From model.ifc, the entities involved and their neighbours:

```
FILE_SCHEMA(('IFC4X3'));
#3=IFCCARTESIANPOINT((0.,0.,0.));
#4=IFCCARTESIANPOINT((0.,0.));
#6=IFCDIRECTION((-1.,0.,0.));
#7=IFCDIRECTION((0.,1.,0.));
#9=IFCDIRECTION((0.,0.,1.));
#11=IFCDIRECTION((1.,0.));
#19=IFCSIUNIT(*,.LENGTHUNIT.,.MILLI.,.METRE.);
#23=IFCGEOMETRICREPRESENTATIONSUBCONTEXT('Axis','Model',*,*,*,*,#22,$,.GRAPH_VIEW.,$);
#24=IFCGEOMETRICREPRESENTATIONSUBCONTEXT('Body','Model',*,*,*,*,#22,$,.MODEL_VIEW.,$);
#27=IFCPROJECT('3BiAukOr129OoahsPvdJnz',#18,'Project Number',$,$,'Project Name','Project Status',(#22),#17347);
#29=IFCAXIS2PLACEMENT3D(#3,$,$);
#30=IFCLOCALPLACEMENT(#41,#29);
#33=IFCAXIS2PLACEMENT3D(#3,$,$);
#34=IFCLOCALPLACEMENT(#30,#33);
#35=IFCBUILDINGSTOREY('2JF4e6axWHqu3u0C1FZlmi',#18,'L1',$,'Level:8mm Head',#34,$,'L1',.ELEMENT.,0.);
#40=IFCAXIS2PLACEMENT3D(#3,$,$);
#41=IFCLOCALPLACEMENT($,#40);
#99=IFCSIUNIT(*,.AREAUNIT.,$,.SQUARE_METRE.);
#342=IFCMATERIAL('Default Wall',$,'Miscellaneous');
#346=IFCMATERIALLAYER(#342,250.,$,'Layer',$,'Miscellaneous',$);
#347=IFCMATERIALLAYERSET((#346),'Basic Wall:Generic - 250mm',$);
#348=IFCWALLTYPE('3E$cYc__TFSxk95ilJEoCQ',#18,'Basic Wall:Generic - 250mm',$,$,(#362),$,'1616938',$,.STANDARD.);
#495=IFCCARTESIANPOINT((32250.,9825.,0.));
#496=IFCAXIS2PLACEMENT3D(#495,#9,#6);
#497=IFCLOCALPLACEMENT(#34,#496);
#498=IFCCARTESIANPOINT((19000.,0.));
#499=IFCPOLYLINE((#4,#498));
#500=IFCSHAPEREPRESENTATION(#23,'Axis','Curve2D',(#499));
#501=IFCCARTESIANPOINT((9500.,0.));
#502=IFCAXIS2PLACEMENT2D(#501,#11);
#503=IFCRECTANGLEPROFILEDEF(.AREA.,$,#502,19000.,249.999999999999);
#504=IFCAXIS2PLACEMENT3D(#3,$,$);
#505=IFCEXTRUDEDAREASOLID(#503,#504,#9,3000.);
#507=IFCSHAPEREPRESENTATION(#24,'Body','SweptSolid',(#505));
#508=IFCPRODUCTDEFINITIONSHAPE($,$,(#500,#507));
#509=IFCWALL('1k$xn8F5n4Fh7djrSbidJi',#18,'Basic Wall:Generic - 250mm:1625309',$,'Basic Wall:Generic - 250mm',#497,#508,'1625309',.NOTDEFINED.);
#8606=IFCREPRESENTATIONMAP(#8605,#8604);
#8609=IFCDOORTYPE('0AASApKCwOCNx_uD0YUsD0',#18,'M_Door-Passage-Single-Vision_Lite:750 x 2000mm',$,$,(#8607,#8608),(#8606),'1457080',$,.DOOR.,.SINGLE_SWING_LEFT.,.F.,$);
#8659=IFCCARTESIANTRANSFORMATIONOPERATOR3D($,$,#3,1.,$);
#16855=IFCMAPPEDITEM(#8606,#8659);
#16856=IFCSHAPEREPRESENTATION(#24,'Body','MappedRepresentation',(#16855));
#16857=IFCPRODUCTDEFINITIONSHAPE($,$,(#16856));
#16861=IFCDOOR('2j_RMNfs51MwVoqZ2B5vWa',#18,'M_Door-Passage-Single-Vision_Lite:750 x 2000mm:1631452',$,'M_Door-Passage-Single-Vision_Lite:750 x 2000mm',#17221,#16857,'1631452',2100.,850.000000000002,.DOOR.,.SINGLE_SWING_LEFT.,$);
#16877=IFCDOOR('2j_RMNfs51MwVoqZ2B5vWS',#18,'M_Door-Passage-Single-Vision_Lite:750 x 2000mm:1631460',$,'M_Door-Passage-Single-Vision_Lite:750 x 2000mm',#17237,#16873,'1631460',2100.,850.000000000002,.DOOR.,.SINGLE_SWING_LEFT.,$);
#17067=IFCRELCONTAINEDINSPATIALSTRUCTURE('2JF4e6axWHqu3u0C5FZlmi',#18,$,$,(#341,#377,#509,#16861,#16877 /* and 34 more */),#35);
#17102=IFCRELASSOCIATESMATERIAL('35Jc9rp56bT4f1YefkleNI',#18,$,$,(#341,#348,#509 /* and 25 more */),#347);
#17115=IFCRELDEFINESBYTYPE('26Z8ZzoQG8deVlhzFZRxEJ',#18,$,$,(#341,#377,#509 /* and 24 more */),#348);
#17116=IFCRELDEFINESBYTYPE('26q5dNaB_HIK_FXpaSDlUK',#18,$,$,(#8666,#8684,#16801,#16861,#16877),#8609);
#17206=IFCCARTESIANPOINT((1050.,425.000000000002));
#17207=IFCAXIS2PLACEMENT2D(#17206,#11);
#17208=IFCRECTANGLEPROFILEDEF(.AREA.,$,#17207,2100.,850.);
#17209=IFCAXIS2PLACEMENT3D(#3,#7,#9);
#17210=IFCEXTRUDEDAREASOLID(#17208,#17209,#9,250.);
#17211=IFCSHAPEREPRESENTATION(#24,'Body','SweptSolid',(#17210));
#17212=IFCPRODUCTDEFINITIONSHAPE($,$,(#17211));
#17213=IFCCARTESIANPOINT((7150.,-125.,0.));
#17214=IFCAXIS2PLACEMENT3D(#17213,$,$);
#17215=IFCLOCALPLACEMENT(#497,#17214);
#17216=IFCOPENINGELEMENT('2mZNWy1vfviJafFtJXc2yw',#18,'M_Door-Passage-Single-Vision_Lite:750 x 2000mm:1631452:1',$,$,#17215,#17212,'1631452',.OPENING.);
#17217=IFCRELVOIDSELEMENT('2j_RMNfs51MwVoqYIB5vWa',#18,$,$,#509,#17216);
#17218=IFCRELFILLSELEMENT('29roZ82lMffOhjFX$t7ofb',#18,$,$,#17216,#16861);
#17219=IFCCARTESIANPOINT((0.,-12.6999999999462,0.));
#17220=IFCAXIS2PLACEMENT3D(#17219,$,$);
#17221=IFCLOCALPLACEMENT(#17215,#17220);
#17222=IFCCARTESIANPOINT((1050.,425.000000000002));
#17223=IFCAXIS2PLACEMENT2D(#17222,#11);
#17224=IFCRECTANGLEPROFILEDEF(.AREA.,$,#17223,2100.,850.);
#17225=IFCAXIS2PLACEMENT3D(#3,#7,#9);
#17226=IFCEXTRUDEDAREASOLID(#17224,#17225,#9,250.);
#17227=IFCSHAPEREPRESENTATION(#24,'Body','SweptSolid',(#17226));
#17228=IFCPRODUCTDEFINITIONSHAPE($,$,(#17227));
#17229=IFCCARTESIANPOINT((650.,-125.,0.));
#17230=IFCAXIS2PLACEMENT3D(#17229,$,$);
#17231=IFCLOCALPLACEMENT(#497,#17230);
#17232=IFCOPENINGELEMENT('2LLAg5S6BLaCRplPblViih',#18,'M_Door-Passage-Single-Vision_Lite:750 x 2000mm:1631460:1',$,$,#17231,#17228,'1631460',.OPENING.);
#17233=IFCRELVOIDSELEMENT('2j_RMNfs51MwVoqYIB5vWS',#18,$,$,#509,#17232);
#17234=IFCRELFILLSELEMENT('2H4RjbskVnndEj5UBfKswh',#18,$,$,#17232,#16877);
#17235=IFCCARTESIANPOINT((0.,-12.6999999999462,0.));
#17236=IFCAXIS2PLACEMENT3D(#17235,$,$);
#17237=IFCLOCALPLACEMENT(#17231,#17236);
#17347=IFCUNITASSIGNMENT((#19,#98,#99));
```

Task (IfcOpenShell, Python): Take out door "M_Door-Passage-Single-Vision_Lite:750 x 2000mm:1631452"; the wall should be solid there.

```python
import ifcopenshell
import ifcopenshell.api.feature
import ifcopenshell.api.root
import ifcopenshell.geom
import ifcopenshell.util.shape

model = ifcopenshell.open("model.ifc")
settings = ifcopenshell.geom.settings()


def volume(element):
    """Net volume in cubic metres, openings subtracted."""
    shape = ifcopenshell.geom.create_shape(settings, element)
    return ifcopenshell.util.shape.get_volume(shape.geometry)


door = model.by_id(16861)
opening = door.FillsVoids[0].RelatingOpeningElement
wall = opening.VoidsElements[0].RelatingBuildingElement
before = volume(wall)

ifcopenshell.api.root.remove_product(model, product=door)
ifcopenshell.api.feature.remove_feature(model, feature=opening)

after = volume(wall)

print(f"wall volume {before:.3f} -> {after:.3f} m3")

model.write("model_v2.ifc")
```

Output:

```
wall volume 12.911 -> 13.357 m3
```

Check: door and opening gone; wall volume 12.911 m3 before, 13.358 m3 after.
